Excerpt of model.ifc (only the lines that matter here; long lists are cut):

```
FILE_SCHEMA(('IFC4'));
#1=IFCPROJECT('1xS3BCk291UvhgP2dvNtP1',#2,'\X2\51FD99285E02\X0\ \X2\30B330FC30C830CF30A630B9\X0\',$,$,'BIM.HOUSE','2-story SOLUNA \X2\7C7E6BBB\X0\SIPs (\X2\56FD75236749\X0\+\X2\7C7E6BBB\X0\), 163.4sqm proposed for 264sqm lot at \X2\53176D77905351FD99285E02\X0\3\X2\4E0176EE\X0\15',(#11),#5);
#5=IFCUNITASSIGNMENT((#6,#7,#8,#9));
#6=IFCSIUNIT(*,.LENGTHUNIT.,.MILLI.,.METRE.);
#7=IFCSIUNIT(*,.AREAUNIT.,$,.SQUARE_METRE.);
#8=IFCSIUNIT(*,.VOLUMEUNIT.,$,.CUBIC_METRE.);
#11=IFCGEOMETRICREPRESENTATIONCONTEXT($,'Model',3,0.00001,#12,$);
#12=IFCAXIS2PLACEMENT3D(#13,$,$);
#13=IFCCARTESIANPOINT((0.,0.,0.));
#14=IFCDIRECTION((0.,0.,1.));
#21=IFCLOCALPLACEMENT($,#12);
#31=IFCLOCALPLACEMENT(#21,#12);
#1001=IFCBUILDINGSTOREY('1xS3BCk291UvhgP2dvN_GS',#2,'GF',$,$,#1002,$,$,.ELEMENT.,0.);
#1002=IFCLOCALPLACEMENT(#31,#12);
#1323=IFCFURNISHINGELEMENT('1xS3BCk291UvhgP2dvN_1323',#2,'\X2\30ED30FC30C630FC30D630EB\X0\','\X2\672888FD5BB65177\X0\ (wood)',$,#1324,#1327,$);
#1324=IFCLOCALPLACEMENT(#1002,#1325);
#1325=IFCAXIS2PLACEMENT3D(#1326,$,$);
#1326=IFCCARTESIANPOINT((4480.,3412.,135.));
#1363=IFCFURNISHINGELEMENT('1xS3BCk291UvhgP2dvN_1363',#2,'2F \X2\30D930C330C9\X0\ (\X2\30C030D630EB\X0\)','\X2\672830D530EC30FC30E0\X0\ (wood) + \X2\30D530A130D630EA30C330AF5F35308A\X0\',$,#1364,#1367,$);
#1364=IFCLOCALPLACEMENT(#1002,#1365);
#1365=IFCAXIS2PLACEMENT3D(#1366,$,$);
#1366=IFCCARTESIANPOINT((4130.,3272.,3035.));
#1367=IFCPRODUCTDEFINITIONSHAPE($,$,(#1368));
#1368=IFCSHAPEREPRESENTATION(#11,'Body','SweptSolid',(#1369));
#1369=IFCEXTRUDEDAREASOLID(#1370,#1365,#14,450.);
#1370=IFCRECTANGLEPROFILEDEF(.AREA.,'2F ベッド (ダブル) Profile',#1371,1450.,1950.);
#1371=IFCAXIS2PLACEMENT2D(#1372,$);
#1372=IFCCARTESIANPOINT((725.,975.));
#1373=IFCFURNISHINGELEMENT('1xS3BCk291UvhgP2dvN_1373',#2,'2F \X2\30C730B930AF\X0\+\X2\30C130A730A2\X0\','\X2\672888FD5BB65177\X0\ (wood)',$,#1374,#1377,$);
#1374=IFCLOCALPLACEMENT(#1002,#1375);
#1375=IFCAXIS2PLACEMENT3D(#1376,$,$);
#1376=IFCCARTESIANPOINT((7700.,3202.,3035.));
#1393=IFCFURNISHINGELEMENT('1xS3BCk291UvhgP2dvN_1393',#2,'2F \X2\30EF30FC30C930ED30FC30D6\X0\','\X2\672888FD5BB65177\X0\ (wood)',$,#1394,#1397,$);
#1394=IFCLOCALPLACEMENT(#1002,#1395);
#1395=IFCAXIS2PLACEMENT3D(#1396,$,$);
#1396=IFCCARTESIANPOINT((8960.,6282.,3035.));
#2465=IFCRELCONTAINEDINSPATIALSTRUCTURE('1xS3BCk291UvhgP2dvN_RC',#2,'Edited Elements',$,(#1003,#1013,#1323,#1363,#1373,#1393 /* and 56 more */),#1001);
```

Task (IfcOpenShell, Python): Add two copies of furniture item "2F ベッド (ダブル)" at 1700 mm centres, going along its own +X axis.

```python
import ifcopenshell
import ifcopenshell.api.geometry
import ifcopenshell.api.root
import ifcopenshell.util.element
import ifcopenshell.util.placement
import ifcopenshell.util.unit

model = ifcopenshell.open("model.ifc")
unit_scale = ifcopenshell.util.unit.calculate_unit_scale(model)


def reuse_history(source, copy):
    """copy_class also copies each property set's owner history, people and application; keep the originals."""
    for rel in copy.IsDefinedBy:
        if rel.is_a("IfcRelDefinesByProperties") and (history := rel.RelatingPropertyDefinition.OwnerHistory):
            rel.RelatingPropertyDefinition.OwnerHistory = source.OwnerHistory
            ifcopenshell.util.element.remove_deep2(model, history)


source = model.by_id(1363)
base = ifcopenshell.util.placement.get_local_placement(source.ObjectPlacement)
step = base[:3, 0] * 1.7 / unit_scale

for i in range(1, 3):
    copy = ifcopenshell.api.root.copy_class(model, product=source)
    copy.Representation = ifcopenshell.util.element.copy_deep(
        model, source.Representation, exclude=["IfcGeometricRepresentationContext", "IfcRepresentationMap"]
    )
    reuse_history(source, copy)
    matrix = base.copy()
    matrix[:3, 3] += i * step
    print("added at", matrix[:3, 3].round(3) + 0.0)
    ifcopenshell.api.geometry.edit_object_placement(model, product=copy, matrix=matrix, is_si=False)

model.write("model_edited.ifc")
```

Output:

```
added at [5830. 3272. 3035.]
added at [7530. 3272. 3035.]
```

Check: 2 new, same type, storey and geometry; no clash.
